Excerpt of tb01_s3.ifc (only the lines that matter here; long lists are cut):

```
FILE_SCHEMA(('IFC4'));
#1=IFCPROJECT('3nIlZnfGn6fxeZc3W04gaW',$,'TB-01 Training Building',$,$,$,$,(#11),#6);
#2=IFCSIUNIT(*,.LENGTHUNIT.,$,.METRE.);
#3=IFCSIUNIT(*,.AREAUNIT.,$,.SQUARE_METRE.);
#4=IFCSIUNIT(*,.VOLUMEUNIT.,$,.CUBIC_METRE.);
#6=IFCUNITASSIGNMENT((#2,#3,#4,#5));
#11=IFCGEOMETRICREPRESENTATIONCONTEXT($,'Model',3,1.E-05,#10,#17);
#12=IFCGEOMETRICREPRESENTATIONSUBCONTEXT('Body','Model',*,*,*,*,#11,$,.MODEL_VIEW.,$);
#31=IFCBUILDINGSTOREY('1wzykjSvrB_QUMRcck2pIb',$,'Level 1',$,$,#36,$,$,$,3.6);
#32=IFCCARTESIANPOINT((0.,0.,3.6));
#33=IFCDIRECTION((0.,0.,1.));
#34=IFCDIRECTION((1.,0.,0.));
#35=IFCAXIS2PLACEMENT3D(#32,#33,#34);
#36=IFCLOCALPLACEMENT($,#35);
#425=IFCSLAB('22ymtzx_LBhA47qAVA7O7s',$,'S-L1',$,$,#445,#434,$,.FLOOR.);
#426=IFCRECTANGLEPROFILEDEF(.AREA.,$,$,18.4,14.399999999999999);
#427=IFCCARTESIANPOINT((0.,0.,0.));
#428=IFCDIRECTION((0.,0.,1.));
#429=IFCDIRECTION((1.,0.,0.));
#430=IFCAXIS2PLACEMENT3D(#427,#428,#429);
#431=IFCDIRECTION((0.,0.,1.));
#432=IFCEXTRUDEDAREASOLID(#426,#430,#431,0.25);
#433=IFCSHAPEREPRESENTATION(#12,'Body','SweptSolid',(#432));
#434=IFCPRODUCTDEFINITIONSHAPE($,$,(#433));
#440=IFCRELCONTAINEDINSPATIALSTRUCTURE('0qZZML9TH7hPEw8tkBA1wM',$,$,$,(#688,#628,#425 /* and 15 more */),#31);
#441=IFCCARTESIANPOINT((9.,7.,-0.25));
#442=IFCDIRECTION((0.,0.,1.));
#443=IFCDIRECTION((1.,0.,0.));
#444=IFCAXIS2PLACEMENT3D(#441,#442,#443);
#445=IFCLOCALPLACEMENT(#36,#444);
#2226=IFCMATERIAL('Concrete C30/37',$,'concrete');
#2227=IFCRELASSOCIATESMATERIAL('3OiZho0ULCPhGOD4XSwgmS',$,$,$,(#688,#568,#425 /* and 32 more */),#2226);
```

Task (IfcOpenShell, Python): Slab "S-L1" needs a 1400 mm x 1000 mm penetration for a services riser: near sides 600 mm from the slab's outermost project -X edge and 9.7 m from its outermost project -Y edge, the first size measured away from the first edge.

```python
import numpy as np
import ifcopenshell
import ifcopenshell.api.feature
import ifcopenshell.api.geometry
import ifcopenshell.api.root
import ifcopenshell.geom
import ifcopenshell.util.placement
import ifcopenshell.util.representation
import ifcopenshell.util.shape
import ifcopenshell.util.unit

model = ifcopenshell.open("tb01_s3.ifc")
unit_scale = ifcopenshell.util.unit.calculate_unit_scale(model)
settings = ifcopenshell.geom.settings()


def volume(element):
    """Net volume in cubic metres, openings subtracted."""
    shape = ifcopenshell.geom.create_shape(settings, element)
    return ifcopenshell.util.shape.get_volume(shape.geometry)


slab = model.by_guid("22ymtzx_LBhA47qAVA7O7s")
before = volume(slab)

# Extent in the slab's own axes, in metres. The edges named are its -X and -Y sides.
slab_shape = ifcopenshell.geom.create_shape(settings, slab)
vertices = ifcopenshell.util.shape.get_vertices(slab_shape.geometry)
x_min, y_min, bottom = vertices.min(axis=0)
top = vertices[:, 2].max()

opening = ifcopenshell.api.root.create_entity(model, ifc_class="IfcOpeningElement", name="Services riser opening", predefined_type="OPENING")
context = ifcopenshell.util.representation.get_context(model, "Model", "Body", "MODEL_VIEW")
width, depth = 1.4, 1
outline = [(0.0, 0.0), (width, 0.0), (width, depth), (0.0, depth), (0.0, 0.0)]
# Overshoot both faces by 50 mm so the cut is clean.
shape = ifcopenshell.api.geometry.add_slab_representation(
    model, context=context, depth=top - bottom + 0.1, polyline=outline
)
ifcopenshell.api.geometry.assign_representation(model, product=opening, representation=shape)

matrix = ifcopenshell.util.placement.get_local_placement(slab.ObjectPlacement)
matrix[:, 3] = matrix @ np.append(np.array([x_min + 0.6, y_min + 9.7, bottom - 0.05]) / unit_scale, 1.0)
ifcopenshell.api.geometry.edit_object_placement(model, product=opening, matrix=matrix, is_si=False)
ifcopenshell.api.feature.add_feature(model, feature=opening, element=slab)

after = volume(slab)

print(f"slab volume {before:.3f} -> {after:.3f} m3")

model.write("tb01_s3_rev.ifc")
```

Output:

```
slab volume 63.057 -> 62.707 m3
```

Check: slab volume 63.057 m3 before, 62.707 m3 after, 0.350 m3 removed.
